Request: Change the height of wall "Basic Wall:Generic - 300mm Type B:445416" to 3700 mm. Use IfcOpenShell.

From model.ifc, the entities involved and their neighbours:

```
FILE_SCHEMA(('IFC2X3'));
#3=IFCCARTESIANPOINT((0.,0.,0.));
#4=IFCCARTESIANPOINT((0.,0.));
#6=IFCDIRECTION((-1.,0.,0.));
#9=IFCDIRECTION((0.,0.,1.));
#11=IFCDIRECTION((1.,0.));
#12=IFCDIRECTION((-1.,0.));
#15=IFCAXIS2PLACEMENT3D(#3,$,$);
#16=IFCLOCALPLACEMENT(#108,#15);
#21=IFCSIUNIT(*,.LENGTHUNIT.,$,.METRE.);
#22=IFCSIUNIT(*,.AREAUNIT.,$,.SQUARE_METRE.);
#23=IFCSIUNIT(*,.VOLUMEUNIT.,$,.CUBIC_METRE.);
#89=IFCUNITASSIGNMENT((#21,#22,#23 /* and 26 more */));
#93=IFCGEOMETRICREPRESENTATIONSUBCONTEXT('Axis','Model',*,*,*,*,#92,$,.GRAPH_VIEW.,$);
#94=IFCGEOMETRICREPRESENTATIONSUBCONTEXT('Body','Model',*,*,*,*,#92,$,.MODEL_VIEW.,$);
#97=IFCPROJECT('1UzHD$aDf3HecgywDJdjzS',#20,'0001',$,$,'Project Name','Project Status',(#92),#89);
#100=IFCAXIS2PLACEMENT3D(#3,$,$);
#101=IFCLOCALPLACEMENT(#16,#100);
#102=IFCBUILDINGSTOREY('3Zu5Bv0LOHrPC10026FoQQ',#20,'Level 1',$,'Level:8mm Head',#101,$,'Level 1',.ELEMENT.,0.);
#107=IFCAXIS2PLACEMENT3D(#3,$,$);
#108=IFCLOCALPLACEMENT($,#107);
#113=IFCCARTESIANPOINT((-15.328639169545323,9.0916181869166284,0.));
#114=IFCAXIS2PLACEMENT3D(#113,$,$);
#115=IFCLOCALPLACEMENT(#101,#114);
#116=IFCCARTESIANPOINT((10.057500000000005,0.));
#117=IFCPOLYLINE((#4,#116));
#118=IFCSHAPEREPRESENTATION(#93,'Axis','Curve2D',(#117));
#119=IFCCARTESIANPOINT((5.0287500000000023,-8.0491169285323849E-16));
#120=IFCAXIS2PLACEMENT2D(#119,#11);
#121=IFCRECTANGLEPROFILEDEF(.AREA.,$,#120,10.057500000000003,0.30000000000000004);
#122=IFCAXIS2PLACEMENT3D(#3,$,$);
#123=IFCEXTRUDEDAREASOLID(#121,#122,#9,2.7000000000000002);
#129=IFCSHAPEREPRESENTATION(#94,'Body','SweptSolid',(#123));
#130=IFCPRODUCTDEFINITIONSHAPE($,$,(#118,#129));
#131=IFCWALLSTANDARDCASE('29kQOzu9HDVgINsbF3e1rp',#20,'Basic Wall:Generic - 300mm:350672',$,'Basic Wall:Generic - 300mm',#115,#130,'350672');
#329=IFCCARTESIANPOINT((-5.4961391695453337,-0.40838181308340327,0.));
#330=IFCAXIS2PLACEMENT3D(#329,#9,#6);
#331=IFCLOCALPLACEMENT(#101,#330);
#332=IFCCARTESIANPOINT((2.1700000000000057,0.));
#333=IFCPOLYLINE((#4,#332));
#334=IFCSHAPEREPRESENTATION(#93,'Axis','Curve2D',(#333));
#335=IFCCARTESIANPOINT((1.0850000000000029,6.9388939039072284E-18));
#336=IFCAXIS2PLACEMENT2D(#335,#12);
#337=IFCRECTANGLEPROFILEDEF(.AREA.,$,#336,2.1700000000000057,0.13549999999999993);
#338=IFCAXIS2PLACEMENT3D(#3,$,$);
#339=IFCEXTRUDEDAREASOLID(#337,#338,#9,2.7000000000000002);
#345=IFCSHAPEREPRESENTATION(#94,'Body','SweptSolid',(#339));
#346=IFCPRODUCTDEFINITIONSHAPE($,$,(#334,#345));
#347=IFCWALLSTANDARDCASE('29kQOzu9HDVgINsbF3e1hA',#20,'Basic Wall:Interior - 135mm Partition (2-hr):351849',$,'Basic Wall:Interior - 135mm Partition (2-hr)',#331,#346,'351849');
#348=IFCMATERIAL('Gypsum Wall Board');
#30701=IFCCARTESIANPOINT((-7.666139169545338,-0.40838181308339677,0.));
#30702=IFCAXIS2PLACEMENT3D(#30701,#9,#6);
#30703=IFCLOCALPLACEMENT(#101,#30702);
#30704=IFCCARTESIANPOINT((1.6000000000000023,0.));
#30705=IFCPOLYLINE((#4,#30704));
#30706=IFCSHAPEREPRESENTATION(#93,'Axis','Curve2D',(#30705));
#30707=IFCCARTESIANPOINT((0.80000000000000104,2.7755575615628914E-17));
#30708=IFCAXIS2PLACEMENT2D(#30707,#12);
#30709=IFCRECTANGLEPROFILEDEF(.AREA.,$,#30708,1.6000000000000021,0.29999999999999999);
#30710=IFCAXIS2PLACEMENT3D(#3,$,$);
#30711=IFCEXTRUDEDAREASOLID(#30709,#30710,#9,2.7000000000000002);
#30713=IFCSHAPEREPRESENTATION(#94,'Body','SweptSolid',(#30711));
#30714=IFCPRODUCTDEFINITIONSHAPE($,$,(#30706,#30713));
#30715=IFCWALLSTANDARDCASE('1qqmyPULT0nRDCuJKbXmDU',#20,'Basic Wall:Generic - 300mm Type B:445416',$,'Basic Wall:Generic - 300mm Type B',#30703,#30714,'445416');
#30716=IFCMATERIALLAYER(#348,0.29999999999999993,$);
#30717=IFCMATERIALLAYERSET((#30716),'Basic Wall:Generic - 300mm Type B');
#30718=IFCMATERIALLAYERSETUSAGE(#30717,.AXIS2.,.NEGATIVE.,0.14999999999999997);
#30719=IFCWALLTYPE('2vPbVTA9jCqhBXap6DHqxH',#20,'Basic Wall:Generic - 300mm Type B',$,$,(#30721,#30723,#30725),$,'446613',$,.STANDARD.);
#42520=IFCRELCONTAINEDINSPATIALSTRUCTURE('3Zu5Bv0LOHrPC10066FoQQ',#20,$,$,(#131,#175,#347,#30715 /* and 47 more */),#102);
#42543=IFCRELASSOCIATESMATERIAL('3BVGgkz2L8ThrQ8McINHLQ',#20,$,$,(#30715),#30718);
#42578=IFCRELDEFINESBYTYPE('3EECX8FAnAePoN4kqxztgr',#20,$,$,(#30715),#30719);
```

```python
import ifcopenshell
import ifcopenshell.geom
import ifcopenshell.util.representation
import ifcopenshell.util.shape
import ifcopenshell.util.unit

model = ifcopenshell.open("model.ifc")
unit_scale = ifcopenshell.util.unit.calculate_unit_scale(model)
settings = ifcopenshell.geom.settings()


def volume(element):
    """Net volume in cubic metres, openings subtracted."""
    shape = ifcopenshell.geom.create_shape(settings, element)
    return ifcopenshell.util.shape.get_volume(shape.geometry)


wall = model.by_guid("1qqmyPULT0nRDCuJKbXmDU")
before = volume(wall)

body = ifcopenshell.util.representation.get_representation(wall, "Model", "Body")
solid = body.Items[0]
old_height = solid.Depth
solid.Depth = 3.7 / unit_scale
after = volume(wall)

print(f"height {old_height:g} -> {solid.Depth:g}, volume {before:.3f} -> {after:.3f} m3")

model.write("model-out.ifc")
```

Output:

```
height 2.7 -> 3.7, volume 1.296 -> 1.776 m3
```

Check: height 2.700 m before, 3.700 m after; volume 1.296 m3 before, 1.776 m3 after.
